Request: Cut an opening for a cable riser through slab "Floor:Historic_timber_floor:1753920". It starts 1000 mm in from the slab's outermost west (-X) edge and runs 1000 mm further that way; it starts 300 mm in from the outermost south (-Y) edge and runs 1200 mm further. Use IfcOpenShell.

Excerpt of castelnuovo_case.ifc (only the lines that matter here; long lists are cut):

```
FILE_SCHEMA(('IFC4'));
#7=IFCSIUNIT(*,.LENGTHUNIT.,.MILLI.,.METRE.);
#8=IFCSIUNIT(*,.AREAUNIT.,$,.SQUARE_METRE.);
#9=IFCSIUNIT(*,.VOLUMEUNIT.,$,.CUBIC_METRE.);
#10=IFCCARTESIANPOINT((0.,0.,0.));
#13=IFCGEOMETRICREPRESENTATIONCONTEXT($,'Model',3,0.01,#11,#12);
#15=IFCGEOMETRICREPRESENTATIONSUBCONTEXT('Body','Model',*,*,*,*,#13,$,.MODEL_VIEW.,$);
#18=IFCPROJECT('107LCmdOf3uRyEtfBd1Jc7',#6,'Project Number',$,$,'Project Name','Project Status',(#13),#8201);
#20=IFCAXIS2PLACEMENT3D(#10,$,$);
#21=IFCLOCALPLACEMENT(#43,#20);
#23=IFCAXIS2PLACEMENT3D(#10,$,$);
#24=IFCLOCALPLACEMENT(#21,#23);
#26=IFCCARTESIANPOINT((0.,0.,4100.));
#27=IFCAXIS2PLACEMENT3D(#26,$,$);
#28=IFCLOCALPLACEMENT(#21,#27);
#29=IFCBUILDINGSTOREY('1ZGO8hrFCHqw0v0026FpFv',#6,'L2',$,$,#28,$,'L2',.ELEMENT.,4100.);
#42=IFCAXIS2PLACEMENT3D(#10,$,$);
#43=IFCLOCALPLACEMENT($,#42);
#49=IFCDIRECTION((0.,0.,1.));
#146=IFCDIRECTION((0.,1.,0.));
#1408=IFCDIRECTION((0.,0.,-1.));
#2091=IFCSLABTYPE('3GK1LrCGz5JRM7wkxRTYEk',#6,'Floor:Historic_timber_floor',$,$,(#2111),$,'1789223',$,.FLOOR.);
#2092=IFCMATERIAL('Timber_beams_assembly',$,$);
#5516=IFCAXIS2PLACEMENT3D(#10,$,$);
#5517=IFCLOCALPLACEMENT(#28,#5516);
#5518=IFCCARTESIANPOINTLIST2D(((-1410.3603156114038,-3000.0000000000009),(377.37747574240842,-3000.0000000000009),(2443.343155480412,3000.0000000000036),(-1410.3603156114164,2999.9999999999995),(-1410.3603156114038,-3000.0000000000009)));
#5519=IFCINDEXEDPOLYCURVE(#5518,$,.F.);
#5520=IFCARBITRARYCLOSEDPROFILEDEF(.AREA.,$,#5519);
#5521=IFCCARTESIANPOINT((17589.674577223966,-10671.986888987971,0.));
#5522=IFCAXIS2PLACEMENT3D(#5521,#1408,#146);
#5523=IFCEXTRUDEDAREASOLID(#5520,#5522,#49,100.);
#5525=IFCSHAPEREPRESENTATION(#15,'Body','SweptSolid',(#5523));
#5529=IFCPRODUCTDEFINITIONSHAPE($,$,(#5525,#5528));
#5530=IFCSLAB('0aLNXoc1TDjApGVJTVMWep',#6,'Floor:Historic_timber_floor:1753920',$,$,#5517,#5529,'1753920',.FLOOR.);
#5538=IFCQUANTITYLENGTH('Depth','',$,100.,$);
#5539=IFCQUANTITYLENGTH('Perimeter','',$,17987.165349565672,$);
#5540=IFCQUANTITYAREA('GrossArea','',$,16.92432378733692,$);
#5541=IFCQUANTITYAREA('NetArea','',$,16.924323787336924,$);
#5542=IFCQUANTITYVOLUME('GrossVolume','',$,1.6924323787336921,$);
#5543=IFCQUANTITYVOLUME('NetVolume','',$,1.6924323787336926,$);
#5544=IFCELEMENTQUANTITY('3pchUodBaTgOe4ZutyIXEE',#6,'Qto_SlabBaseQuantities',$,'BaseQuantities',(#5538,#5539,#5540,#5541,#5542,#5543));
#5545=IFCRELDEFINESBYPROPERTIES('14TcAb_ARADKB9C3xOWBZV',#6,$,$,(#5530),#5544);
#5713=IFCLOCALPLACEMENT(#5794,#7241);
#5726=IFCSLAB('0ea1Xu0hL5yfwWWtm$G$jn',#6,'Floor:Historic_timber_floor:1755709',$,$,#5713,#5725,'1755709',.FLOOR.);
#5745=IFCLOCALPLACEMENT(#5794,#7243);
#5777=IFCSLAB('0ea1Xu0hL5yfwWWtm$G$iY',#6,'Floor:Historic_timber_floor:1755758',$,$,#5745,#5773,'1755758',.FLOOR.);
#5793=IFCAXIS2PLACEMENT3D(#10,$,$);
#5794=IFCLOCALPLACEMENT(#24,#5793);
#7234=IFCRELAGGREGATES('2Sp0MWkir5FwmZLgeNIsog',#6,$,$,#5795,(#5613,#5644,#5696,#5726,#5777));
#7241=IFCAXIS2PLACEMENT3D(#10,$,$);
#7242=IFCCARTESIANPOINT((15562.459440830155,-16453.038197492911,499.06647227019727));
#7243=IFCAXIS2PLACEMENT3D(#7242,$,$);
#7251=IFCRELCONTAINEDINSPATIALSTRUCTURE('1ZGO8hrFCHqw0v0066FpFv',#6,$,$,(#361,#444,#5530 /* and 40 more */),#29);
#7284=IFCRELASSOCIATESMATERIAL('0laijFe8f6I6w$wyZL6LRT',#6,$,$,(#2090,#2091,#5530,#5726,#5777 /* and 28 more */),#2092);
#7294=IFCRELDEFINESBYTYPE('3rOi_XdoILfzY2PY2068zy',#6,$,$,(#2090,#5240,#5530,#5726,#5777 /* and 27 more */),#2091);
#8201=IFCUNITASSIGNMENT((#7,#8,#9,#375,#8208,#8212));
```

```python
import numpy as np
import ifcopenshell
import ifcopenshell.api.feature
import ifcopenshell.api.geometry
import ifcopenshell.api.pset
import ifcopenshell.api.root
import ifcopenshell.geom
import ifcopenshell.util.element
import ifcopenshell.util.placement
import ifcopenshell.util.representation
import ifcopenshell.util.shape
import ifcopenshell.util.unit

model = ifcopenshell.open("castelnuovo_case.ifc")
unit_scale = ifcopenshell.util.unit.calculate_unit_scale(model)
area_scale = ifcopenshell.util.unit.calculate_unit_scale(model, "AREAUNIT")
volume_scale = ifcopenshell.util.unit.calculate_unit_scale(model, "VOLUMEUNIT")
settings = ifcopenshell.geom.settings()


def volume(element):
    """Net volume in cubic metres, openings subtracted."""
    shape = ifcopenshell.geom.create_shape(settings, element)
    return ifcopenshell.util.shape.get_volume(shape.geometry)


slab = model.by_guid("0aLNXoc1TDjApGVJTVMWep")
before = volume(slab)

# Extent in the slab's own axes, in metres. The edges named are its -X and -Y sides.
slab_shape = ifcopenshell.geom.create_shape(settings, slab)
vertices = ifcopenshell.util.shape.get_vertices(slab_shape.geometry)
x_min, y_min, bottom = vertices.min(axis=0)
top = vertices[:, 2].max()

opening = ifcopenshell.api.root.create_entity(model, ifc_class="IfcOpeningElement", name="Cable riser opening", predefined_type="OPENING")
context = ifcopenshell.util.representation.get_context(model, "Model", "Body", "MODEL_VIEW")
width, depth = 1, 1.2
outline = [(0.0, 0.0), (width, 0.0), (width, depth), (0.0, depth), (0.0, 0.0)]
# Overshoot both faces by 50 mm so the cut is clean.
shape = ifcopenshell.api.geometry.add_slab_representation(
    model, context=context, depth=top - bottom + 0.1, polyline=outline
)
ifcopenshell.api.geometry.assign_representation(model, product=opening, representation=shape)

matrix = ifcopenshell.util.placement.get_local_placement(slab.ObjectPlacement)
matrix[:, 3] = matrix @ np.append(np.array([x_min + 1, y_min + 0.3, bottom - 0.05]) / unit_scale, 1.0)
ifcopenshell.api.geometry.edit_object_placement(model, product=opening, matrix=matrix, is_si=False)
ifcopenshell.api.feature.add_feature(model, feature=opening, element=slab)

after = volume(slab)

# Update the slab's stored quantities.
qto = model.by_id(ifcopenshell.util.element.get_pset(slab, "Qto_SlabBaseQuantities", should_inherit=False)["id"])
ifcopenshell.api.pset.edit_qto(model, qto=qto, properties={
    "NetArea": after / (top - bottom) / area_scale,
    "NetVolume": after / volume_scale,
})

print(f"slab volume {before:.3f} -> {after:.3f} m3")

model.write("castelnuovo_case_updated.ifc")
```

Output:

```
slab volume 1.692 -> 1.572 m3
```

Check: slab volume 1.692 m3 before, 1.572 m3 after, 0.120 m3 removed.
